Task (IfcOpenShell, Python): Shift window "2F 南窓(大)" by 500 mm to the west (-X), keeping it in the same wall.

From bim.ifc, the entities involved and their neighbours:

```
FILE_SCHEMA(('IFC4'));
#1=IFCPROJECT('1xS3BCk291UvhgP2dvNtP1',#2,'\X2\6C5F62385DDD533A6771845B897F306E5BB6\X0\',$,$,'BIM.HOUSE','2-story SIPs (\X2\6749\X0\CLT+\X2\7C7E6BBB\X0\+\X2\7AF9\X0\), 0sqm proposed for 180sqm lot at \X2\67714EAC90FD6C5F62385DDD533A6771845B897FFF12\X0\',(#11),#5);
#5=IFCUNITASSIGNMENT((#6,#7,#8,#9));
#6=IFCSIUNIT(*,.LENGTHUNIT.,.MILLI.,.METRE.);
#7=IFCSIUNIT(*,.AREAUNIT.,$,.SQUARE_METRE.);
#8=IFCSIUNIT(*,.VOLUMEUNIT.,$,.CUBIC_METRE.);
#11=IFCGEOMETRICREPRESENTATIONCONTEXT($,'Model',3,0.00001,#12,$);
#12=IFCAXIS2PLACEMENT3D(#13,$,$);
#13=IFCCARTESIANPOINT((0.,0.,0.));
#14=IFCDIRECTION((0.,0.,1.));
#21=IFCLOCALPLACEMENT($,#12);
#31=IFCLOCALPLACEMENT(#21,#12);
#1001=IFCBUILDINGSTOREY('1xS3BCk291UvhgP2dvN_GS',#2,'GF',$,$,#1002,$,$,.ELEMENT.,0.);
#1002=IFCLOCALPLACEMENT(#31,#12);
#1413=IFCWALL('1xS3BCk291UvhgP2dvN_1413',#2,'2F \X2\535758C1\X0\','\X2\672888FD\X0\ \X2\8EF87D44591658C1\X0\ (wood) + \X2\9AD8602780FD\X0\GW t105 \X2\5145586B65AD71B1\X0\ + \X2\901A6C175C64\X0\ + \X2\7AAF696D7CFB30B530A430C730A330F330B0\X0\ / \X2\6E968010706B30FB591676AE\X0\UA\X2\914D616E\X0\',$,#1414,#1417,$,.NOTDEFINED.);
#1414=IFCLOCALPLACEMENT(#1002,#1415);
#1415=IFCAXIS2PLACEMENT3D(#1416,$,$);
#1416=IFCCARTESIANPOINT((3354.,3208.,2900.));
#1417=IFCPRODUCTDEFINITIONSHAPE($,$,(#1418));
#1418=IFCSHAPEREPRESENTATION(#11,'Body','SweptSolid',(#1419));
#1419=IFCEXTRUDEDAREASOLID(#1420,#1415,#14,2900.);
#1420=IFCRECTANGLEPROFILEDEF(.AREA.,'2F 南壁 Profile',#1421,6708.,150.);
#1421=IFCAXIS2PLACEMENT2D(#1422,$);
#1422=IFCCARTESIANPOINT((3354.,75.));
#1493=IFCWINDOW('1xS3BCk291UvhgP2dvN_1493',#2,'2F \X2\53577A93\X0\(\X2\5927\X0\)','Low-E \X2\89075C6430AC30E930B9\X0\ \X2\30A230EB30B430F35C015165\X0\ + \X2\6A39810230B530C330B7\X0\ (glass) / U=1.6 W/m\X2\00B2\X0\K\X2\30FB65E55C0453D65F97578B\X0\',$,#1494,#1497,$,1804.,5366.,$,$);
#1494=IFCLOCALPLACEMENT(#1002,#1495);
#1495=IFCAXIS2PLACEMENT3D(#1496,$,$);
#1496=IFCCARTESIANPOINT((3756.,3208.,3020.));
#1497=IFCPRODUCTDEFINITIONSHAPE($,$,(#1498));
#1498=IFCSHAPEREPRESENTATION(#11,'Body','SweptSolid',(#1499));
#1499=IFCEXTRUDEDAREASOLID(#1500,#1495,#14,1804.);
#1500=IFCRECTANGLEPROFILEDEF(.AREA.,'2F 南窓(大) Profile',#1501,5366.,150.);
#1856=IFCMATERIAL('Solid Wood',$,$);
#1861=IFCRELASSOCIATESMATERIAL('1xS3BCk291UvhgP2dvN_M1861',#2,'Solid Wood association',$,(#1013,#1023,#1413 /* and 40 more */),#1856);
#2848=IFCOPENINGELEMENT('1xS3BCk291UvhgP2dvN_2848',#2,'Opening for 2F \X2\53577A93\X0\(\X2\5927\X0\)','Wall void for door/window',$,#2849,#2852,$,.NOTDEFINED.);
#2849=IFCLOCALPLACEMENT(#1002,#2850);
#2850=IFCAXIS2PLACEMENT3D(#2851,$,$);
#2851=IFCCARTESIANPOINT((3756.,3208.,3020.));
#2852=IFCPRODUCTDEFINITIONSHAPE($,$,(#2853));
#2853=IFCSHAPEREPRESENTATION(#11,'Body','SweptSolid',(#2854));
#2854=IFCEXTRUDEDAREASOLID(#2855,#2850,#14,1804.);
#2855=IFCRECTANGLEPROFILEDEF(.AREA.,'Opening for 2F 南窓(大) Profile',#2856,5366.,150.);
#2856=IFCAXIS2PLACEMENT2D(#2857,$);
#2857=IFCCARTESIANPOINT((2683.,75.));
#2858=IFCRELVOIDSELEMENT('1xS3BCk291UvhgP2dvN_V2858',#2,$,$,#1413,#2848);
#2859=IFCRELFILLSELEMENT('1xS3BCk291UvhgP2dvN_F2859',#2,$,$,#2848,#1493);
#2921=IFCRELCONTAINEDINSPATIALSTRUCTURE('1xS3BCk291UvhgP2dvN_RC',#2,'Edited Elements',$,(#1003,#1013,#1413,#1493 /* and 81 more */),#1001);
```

```python
import ifcopenshell
import ifcopenshell.api.geometry
import ifcopenshell.util.placement

model = ifcopenshell.open("bim.ifc")

window = model.by_guid("1xS3BCk291UvhgP2dvN_1493")
opening = window.FillsVoids[0].RelatingOpeningElement
wall = opening.VoidsElements[0].RelatingBuildingElement

wall_matrix = ifcopenshell.util.placement.get_local_placement(wall.ObjectPlacement)
shift = wall_matrix[:3, 0] * -500.0
before = ifcopenshell.util.placement.get_local_placement(window.ObjectPlacement)[:3, 3].copy()

# The window is not placed relative to its opening, so move both.
for product in (opening, window):
    matrix = ifcopenshell.util.placement.get_local_placement(product.ObjectPlacement)
    matrix[:3, 3] += shift
    ifcopenshell.api.geometry.edit_object_placement(model, product=product, matrix=matrix, is_si=False)

after = ifcopenshell.util.placement.get_local_placement(window.ObjectPlacement)[:3, 3]
print("window moved by", (after - before).round(3) + 0.0)

model.write("bim_updated.ifc")
```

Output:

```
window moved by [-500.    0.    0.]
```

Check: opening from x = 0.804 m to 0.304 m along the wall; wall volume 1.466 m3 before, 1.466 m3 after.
